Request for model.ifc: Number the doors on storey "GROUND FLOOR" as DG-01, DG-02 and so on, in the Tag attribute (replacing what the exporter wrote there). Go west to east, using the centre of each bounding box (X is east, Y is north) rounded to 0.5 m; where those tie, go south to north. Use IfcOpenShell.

First a look at what the model holds.

```python
import ifcopenshell
import ifcopenshell.util.element
import ifcopenshell.util.placement

model = ifcopenshell.open("model.ifc")
print(model.schema)
storey = next(s for s in model.by_type("IfcBuildingStorey") if s.Name == "GROUND FLOOR")
doors = [e for e in ifcopenshell.util.element.get_decomposition(storey) if e.is_a("IfcDoor")]
for e in sorted(doors, key=lambda e: e.id()):
    origin = ifcopenshell.util.placement.get_local_placement(e.ObjectPlacement)[:3, 3]
    print(e.id(), e.Tag, e.Name, origin.round(2) + 0.0, sep=" | ")
```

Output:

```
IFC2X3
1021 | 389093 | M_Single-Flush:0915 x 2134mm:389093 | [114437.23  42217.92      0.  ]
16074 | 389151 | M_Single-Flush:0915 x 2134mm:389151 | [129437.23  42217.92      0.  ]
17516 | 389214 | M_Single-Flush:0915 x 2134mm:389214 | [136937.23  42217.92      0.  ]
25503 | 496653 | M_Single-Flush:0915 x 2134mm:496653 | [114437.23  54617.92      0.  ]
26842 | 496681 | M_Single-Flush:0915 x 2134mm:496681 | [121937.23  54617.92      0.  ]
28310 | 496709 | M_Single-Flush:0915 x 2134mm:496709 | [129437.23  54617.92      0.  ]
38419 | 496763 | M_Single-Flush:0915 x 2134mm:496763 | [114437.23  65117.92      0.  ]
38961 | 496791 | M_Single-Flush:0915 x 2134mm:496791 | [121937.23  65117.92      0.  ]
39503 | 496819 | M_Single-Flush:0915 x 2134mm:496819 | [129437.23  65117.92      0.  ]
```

```python
import ifcopenshell
import ifcopenshell.geom
import ifcopenshell.util.element
import ifcopenshell.util.shape

model = ifcopenshell.open("model.ifc")
settings = ifcopenshell.geom.settings()
settings.set("use-world-coords", True)


def centre(element):
    shape = ifcopenshell.geom.create_shape(settings, element)
    return ifcopenshell.util.shape.get_bbox_centroid(shape.geometry)


storey = next(s for s in model.by_type("IfcBuildingStorey") if s.Name == "GROUND FLOOR")
doors = [e for e in ifcopenshell.util.element.get_decomposition(storey) if e.is_a("IfcDoor")]

# Insertion points can sit at a corner or the storey origin, so sort by the geometry (in metres).
centres = {e: centre(e) for e in doors}
doors.sort(key=lambda e: (round(centres[e][0] / 0.5), centres[e][1]))

for i, e in enumerate(doors, start=1):
    number = f"DG-{i:02d}"
    e.Tag = number
    print(e.id(), number)

model.write("model_edited.ifc")
```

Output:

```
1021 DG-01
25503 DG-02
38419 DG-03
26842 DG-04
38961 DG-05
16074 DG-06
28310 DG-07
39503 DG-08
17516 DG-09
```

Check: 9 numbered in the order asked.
